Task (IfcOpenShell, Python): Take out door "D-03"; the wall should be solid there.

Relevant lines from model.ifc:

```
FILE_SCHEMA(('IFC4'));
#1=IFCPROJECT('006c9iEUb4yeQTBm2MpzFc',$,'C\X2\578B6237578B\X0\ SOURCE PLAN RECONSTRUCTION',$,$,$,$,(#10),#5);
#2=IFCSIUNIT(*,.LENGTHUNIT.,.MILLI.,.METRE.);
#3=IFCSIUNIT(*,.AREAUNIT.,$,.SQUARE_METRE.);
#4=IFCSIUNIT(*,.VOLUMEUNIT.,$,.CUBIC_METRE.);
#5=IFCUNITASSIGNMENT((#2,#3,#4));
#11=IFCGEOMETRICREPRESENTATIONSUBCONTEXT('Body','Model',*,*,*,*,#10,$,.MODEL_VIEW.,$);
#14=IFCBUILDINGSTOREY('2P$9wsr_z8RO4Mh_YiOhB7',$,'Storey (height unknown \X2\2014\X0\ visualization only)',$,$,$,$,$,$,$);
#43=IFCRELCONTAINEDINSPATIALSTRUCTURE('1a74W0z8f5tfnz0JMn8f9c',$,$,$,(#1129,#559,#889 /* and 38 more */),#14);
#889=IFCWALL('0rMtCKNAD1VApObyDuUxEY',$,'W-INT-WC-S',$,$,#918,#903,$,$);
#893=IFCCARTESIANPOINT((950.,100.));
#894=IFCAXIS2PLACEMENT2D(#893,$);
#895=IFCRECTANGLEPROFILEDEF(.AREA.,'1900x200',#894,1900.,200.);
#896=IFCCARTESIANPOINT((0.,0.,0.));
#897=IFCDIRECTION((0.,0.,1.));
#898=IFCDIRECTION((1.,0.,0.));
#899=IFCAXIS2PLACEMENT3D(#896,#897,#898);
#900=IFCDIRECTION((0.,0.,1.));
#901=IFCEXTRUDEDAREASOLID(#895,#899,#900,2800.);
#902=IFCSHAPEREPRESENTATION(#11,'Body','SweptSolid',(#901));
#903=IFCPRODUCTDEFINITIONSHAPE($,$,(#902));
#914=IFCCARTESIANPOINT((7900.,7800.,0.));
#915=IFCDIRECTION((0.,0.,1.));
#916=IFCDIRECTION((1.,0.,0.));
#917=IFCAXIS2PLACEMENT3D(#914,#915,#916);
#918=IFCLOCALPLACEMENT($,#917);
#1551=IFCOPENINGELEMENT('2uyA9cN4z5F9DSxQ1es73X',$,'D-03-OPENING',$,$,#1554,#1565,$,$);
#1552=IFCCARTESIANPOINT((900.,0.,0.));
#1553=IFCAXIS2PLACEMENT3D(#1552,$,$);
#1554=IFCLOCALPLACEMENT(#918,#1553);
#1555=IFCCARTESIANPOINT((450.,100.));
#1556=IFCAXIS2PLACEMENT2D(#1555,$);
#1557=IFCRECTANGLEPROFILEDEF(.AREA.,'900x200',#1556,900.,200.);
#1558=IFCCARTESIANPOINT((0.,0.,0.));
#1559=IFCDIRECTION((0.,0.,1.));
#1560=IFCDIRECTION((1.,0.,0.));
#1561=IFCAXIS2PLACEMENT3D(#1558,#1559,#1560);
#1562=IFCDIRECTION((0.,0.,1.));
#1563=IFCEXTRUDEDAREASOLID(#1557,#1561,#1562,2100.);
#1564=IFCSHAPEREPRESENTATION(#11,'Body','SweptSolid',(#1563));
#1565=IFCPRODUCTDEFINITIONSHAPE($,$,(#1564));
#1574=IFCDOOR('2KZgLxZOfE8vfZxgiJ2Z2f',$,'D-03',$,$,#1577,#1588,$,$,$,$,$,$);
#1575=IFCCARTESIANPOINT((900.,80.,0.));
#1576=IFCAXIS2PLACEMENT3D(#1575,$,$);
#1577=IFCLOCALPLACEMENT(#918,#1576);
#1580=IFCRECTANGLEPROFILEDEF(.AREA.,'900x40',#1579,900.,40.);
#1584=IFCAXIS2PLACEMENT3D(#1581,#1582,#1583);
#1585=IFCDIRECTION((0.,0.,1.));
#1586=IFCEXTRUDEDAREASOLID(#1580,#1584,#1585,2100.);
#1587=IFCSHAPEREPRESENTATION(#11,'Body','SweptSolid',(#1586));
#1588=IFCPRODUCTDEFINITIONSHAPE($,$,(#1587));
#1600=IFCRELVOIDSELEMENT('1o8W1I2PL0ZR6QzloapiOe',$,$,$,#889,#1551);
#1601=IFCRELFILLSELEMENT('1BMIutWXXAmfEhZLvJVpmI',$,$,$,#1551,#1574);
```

```python
import ifcopenshell
import ifcopenshell.api.feature
import ifcopenshell.api.root
import ifcopenshell.geom
import ifcopenshell.util.shape

model = ifcopenshell.open("model.ifc")
settings = ifcopenshell.geom.settings()


def volume(element):
    """Net volume in cubic metres, openings subtracted."""
    shape = ifcopenshell.geom.create_shape(settings, element)
    return ifcopenshell.util.shape.get_volume(shape.geometry)


door = model.by_guid("2KZgLxZOfE8vfZxgiJ2Z2f")
opening = door.FillsVoids[0].RelatingOpeningElement
wall = opening.VoidsElements[0].RelatingBuildingElement
before = volume(wall)

ifcopenshell.api.root.remove_product(model, product=door)
ifcopenshell.api.feature.remove_feature(model, feature=opening)

after = volume(wall)

print(f"wall volume {before:.3f} -> {after:.3f} m3")

model.write("model_rev.ifc")
```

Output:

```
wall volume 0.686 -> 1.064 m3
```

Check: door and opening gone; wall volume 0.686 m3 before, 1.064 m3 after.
